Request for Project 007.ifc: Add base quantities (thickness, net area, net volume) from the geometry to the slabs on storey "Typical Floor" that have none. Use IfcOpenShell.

First a look at what the model holds.

```python
import ifcopenshell
import ifcopenshell.util.element
import ifcopenshell.util.unit

model = ifcopenshell.open("Project 007.ifc")
print(model.schema)
for unit_type in ("LENGTHUNIT", "AREAUNIT", "VOLUMEUNIT"):
    print(unit_type, ifcopenshell.util.unit.calculate_unit_scale(model, unit_type))
storey = next(s for s in model.by_type("IfcBuildingStorey") if s.Name == "Typical Floor")
slabs = [e for e in ifcopenshell.util.element.get_decomposition(storey) if e.is_a("IfcSlab")]
for e in sorted(slabs, key=lambda e: e.id()):
    print(e.id(), e.is_a(), e.Name, list(ifcopenshell.util.element.get_psets(e, qtos_only=True)), sep=" | ")
```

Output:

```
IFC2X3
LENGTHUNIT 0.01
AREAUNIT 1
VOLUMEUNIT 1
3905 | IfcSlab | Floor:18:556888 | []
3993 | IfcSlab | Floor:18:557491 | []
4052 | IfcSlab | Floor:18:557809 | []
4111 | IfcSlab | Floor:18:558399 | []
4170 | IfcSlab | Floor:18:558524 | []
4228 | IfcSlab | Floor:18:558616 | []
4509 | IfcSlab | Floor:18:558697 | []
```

```python
import ifcopenshell
import ifcopenshell.api.pset
import ifcopenshell.geom
import ifcopenshell.util.element
import ifcopenshell.util.shape
import ifcopenshell.util.unit

model = ifcopenshell.open("Project 007.ifc")
unit_scale = ifcopenshell.util.unit.calculate_unit_scale(model)
area_scale = ifcopenshell.util.unit.calculate_unit_scale(model, "AREAUNIT")
volume_scale = ifcopenshell.util.unit.calculate_unit_scale(model, "VOLUMEUNIT")
settings = ifcopenshell.geom.settings()

storey = next(s for s in model.by_type("IfcBuildingStorey") if s.Name == "Typical Floor")
slabs = [e for e in ifcopenshell.util.element.get_decomposition(storey) if e.is_a("IfcSlab")]

for e in sorted(slabs, key=lambda e: e.id()):
    if ifcopenshell.util.element.get_psets(e, qtos_only=True, should_inherit=False):
        continue
    # Geometry comes back in metres, in the element's own axes.
    shape = ifcopenshell.geom.create_shape(settings, e)
    values = {
        "Width": ifcopenshell.util.shape.get_z(shape.geometry) / unit_scale,
        "NetArea": ifcopenshell.util.shape.get_footprint_area(shape.geometry) / area_scale,
        "NetVolume": ifcopenshell.util.shape.get_volume(shape.geometry) / volume_scale,
    }
    qto = ifcopenshell.api.pset.add_qto(model, product=e, name="BaseQuantities")
    ifcopenshell.api.pset.edit_qto(model, qto=qto, properties=values)
    print(e.id(), {k: round(v, 3) for k, v in values.items()})

model.write("Project 007_updated.ifc")
```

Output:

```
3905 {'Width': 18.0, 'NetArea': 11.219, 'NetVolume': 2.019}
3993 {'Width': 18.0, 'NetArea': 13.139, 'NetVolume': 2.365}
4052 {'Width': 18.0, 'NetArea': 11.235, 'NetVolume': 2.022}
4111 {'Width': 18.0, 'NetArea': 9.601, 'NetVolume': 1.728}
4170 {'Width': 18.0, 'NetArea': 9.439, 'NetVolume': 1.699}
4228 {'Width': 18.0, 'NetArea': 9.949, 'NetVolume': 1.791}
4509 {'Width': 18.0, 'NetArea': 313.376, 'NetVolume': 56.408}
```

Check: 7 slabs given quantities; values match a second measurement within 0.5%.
